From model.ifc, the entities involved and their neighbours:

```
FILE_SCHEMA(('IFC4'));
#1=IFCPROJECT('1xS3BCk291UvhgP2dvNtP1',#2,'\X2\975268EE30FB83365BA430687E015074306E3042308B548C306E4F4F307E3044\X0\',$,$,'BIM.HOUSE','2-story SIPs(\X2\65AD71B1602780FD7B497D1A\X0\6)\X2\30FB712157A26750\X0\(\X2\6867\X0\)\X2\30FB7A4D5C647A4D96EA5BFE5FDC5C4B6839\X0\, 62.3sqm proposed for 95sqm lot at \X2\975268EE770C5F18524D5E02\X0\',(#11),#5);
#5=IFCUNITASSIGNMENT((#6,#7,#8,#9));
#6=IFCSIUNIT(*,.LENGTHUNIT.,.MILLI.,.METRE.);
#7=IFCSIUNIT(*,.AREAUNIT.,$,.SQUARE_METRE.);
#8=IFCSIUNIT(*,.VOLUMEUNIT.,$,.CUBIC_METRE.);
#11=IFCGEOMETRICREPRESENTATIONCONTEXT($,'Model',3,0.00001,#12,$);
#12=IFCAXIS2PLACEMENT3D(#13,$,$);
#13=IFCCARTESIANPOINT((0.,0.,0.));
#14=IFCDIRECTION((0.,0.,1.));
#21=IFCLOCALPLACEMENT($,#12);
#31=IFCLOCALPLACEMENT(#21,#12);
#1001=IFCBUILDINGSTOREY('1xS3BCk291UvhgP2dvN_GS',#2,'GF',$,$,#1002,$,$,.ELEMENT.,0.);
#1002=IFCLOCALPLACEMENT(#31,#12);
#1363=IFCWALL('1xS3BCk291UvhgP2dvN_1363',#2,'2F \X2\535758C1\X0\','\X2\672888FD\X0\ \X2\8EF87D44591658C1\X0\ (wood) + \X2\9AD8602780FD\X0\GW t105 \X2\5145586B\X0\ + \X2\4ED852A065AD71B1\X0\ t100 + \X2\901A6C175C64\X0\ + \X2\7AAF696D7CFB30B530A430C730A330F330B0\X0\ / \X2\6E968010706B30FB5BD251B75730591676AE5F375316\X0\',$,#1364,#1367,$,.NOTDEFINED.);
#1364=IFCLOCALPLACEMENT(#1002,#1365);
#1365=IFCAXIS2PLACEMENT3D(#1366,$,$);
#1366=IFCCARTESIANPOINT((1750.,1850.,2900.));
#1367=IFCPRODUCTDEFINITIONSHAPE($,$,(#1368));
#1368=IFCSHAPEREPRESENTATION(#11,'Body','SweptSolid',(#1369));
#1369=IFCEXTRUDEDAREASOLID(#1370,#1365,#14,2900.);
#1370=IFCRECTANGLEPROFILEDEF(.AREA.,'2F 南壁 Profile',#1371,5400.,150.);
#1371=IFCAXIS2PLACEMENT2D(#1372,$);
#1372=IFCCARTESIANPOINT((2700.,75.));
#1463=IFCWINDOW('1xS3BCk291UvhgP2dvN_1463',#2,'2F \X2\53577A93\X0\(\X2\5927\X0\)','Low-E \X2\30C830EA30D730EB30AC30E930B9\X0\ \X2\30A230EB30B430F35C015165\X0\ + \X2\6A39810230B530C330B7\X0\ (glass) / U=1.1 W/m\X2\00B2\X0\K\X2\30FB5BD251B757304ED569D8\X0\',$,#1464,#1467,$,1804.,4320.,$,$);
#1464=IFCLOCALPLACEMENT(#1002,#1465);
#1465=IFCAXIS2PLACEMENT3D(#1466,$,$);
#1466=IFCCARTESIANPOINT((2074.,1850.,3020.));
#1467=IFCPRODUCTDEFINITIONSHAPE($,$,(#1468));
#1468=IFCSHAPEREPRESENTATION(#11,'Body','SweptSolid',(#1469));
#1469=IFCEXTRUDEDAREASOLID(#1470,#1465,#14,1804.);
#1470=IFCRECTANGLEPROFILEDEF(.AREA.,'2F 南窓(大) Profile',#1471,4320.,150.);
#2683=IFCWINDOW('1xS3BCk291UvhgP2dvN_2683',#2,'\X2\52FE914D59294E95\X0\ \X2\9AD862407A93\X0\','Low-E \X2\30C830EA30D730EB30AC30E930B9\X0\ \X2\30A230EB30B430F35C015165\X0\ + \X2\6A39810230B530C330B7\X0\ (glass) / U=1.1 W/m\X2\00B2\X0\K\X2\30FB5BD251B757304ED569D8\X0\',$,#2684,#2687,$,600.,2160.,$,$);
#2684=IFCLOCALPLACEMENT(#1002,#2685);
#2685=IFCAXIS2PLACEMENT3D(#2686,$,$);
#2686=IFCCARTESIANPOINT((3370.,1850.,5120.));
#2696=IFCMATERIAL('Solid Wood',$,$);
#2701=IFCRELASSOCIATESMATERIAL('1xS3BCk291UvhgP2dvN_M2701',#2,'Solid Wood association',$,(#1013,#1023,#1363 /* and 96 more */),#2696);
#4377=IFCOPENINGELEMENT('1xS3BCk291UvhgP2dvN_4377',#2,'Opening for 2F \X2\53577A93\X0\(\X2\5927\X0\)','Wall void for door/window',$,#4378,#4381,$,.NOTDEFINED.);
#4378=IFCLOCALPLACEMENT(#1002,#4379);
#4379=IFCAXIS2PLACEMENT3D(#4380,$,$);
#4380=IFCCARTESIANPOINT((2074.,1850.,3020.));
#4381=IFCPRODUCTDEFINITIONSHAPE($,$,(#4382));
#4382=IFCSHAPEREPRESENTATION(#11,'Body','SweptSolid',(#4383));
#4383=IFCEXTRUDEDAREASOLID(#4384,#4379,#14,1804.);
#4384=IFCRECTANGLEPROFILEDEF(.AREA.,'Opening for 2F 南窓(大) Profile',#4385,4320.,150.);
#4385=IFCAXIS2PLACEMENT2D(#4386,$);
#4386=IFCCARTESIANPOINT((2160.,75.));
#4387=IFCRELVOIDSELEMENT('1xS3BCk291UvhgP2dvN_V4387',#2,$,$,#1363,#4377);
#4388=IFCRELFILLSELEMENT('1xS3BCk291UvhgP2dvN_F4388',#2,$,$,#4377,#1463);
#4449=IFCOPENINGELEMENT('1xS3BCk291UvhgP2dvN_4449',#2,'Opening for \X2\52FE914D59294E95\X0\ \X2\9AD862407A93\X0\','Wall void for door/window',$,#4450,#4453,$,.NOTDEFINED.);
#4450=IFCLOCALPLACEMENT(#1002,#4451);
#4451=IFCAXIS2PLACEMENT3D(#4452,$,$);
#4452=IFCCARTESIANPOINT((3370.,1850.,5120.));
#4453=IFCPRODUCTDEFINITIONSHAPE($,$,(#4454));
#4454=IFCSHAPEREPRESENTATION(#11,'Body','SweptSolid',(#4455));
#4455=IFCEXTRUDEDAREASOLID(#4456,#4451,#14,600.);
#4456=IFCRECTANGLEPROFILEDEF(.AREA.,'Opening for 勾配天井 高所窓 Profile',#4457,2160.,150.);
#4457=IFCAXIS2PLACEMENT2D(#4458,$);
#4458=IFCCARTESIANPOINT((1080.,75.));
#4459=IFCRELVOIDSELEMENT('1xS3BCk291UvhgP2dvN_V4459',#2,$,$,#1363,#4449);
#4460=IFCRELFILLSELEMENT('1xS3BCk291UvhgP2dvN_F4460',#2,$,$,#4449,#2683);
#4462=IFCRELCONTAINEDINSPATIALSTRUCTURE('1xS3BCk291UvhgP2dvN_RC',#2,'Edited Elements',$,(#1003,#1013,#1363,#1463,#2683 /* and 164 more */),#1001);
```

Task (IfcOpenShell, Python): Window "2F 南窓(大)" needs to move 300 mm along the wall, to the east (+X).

```python
import ifcopenshell
import ifcopenshell.api.geometry
import ifcopenshell.util.placement

model = ifcopenshell.open("model.ifc")

window = model.by_guid("1xS3BCk291UvhgP2dvN_1463")
opening = window.FillsVoids[0].RelatingOpeningElement
wall = opening.VoidsElements[0].RelatingBuildingElement

wall_matrix = ifcopenshell.util.placement.get_local_placement(wall.ObjectPlacement)
shift = wall_matrix[:3, 0] * 300.0
before = ifcopenshell.util.placement.get_local_placement(window.ObjectPlacement)[:3, 3].copy()

# The window is not placed relative to its opening, so move both.
for product in (opening, window):
    matrix = ifcopenshell.util.placement.get_local_placement(product.ObjectPlacement)
    matrix[:3, 3] += shift
    ifcopenshell.api.geometry.edit_object_placement(model, product=product, matrix=matrix, is_si=False)

after = ifcopenshell.util.placement.get_local_placement(window.ObjectPlacement)[:3, 3]
print("window moved by", (after - before).round(3) + 0.0)

model.write("model_updated.ifc")
```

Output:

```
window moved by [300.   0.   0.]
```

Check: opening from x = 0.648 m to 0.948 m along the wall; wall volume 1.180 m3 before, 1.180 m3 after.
